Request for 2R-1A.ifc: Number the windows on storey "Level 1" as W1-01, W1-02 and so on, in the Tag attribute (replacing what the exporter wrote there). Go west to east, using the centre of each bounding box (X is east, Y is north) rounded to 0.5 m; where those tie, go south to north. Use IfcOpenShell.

First a look at what the model holds.

```python
import ifcopenshell
import ifcopenshell.util.element
import ifcopenshell.util.placement

model = ifcopenshell.open("2R-1A.ifc")
print(model.schema)
storey = next(s for s in model.by_type("IfcBuildingStorey") if s.Name == "Level 1")
windows = [e for e in ifcopenshell.util.element.get_decomposition(storey) if e.is_a("IfcWindow")]
for e in sorted(windows, key=lambda e: e.id()):
    origin = ifcopenshell.util.placement.get_local_placement(e.ObjectPlacement)[:3, 3]
    print(e.id(), e.Tag, e.Name, origin.round(2) + 0.0, sep=" | ")
```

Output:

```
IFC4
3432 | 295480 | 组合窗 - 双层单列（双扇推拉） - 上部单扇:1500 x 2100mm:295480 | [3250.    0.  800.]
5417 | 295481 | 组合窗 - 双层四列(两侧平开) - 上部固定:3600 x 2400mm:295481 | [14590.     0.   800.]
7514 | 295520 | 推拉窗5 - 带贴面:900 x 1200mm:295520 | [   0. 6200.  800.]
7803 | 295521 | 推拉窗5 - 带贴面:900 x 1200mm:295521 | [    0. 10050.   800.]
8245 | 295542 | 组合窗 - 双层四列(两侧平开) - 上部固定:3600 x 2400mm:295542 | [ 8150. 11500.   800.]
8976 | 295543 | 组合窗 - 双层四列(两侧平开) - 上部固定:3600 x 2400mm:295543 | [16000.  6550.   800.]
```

```python
import ifcopenshell
import ifcopenshell.geom
import ifcopenshell.util.element
import ifcopenshell.util.shape

model = ifcopenshell.open("2R-1A.ifc")
settings = ifcopenshell.geom.settings()
settings.set("use-world-coords", True)


def centre(element):
    shape = ifcopenshell.geom.create_shape(settings, element)
    return ifcopenshell.util.shape.get_bbox_centroid(shape.geometry)


storey = next(s for s in model.by_type("IfcBuildingStorey") if s.Name == "Level 1")
windows = [e for e in ifcopenshell.util.element.get_decomposition(storey) if e.is_a("IfcWindow")]

# Insertion points can sit at a corner or the storey origin, so sort by the geometry (in metres).
centres = {e: centre(e) for e in windows}
windows.sort(key=lambda e: (round(centres[e][0] / 0.5), centres[e][1]))

for i, e in enumerate(windows, start=1):
    number = f"W1-{i:02d}"
    e.Tag = number
    print(e.id(), number)

model.write("2R-1A_edited.ifc")
```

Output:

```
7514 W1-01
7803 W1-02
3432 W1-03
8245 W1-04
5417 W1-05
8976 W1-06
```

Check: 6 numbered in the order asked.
